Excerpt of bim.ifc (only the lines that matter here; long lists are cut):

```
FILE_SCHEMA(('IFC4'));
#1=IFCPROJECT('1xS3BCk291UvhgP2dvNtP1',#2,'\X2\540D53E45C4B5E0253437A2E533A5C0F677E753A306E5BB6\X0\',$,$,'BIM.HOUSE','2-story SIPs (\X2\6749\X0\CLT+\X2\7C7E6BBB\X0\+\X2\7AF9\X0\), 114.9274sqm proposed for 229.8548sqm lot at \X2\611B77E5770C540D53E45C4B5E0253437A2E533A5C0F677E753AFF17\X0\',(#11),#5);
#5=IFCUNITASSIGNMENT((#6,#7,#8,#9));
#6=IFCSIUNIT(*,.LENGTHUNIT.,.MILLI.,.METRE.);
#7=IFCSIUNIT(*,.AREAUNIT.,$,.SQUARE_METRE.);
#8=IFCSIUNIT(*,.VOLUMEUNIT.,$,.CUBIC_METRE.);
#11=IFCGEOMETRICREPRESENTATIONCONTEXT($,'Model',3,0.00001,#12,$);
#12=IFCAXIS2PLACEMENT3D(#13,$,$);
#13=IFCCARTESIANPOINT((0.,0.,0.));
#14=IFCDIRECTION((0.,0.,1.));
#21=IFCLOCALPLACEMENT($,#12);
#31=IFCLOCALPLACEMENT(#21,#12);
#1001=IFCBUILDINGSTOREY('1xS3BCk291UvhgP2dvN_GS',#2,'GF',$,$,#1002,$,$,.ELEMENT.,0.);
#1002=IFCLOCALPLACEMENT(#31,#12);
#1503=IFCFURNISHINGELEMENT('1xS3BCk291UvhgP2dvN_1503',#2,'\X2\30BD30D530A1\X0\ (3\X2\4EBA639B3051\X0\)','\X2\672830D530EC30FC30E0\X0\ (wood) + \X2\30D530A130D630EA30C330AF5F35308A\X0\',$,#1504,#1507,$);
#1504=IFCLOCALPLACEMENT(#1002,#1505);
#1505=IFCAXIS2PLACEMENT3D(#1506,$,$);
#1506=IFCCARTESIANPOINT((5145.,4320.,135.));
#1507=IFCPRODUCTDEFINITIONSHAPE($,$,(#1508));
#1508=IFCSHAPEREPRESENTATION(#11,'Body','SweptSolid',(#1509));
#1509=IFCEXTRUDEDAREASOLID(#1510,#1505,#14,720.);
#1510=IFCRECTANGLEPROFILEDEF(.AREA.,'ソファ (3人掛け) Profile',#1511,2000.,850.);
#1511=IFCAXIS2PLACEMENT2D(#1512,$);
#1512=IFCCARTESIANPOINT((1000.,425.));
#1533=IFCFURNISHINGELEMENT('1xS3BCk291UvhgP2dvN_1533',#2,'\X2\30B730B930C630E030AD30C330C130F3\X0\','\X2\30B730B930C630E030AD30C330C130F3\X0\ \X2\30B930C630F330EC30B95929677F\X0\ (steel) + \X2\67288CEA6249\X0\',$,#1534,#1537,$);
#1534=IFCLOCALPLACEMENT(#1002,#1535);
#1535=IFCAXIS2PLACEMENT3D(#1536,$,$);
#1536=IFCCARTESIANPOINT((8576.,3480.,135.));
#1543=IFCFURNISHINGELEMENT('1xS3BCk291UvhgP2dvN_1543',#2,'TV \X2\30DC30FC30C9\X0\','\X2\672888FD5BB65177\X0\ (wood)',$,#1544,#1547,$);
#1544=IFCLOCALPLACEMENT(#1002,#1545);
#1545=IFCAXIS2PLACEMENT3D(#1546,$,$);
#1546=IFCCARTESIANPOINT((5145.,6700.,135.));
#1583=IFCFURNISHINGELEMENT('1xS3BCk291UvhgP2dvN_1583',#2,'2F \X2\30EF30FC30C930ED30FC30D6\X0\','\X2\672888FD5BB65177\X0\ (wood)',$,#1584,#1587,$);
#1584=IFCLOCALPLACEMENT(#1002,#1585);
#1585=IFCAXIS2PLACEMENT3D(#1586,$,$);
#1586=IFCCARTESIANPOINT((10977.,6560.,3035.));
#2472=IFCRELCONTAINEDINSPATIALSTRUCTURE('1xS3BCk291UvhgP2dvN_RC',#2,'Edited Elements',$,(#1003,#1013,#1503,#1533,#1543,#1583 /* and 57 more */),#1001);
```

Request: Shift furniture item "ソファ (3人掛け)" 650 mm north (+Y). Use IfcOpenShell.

```python
import ifcopenshell
import ifcopenshell.api.geometry
import ifcopenshell.util.placement
import ifcopenshell.util.unit

model = ifcopenshell.open("bim.ifc")
unit_scale = ifcopenshell.util.unit.calculate_unit_scale(model)

item = model.by_id(1503)
matrix = ifcopenshell.util.placement.get_local_placement(item.ObjectPlacement)
matrix[1, 3] += 0.65 / unit_scale
ifcopenshell.api.geometry.edit_object_placement(model, product=item, matrix=matrix, is_si=False)

print(ifcopenshell.util.placement.get_local_placement(item.ObjectPlacement).round(3) + 0.0)

model.write("bim_rev.ifc")
```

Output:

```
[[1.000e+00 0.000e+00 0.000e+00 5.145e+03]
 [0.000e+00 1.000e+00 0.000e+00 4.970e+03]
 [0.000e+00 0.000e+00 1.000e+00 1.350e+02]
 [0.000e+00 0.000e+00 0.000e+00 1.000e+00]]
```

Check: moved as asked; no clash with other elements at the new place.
